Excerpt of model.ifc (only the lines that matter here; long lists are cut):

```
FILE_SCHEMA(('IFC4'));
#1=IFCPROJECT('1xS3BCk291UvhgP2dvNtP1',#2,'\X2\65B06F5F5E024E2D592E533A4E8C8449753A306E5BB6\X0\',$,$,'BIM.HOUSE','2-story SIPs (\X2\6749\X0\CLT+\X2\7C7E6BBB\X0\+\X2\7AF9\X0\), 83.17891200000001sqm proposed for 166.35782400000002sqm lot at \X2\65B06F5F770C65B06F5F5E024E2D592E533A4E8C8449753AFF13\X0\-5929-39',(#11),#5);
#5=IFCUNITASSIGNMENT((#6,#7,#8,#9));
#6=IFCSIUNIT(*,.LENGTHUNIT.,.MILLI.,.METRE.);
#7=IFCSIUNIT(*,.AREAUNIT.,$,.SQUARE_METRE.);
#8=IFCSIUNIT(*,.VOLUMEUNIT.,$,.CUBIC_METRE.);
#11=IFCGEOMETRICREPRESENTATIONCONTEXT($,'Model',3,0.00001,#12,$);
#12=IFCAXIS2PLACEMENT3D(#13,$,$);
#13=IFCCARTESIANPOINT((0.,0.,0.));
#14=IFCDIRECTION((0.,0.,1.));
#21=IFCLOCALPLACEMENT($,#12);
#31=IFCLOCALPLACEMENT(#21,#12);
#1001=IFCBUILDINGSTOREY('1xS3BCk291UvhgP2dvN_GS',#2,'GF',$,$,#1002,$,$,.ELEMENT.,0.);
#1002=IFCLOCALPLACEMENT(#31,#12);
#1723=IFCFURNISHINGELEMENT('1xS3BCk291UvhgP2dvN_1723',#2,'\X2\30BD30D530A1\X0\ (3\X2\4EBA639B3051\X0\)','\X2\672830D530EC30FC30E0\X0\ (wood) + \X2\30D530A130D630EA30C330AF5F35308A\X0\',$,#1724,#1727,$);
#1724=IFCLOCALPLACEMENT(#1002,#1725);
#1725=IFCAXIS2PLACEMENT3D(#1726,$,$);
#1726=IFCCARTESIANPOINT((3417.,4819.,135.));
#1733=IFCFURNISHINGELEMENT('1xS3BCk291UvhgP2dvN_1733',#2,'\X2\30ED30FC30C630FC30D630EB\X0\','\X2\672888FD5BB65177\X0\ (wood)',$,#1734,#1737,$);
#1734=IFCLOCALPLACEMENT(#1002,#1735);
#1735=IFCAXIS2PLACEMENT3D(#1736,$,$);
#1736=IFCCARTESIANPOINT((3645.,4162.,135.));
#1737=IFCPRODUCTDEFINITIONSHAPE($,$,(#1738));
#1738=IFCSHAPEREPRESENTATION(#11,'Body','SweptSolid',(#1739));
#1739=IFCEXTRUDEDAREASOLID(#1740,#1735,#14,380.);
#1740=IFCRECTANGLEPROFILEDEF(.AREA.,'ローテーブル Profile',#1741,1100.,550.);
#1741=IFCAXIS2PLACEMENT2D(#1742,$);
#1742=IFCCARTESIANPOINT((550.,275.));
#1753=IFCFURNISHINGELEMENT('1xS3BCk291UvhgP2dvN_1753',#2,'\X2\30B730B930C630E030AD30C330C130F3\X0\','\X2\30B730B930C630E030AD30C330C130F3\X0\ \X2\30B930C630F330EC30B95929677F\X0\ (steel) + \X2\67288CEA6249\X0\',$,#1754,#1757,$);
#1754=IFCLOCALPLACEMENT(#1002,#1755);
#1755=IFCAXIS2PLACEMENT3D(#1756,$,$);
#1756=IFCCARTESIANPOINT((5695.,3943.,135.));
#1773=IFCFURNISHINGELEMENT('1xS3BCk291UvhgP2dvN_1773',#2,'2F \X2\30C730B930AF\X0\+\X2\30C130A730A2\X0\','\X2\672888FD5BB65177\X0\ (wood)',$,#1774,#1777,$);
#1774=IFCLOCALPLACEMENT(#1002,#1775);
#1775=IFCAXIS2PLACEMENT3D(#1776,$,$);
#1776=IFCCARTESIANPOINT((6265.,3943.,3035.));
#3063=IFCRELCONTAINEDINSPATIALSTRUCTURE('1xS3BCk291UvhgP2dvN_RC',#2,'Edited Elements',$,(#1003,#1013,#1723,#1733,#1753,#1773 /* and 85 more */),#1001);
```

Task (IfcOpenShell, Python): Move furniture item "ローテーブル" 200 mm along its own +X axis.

```python
import ifcopenshell
import ifcopenshell.api.geometry
import ifcopenshell.util.placement

model = ifcopenshell.open("model.ifc")

item = model.by_id(1733)
matrix = ifcopenshell.util.placement.get_local_placement(item.ObjectPlacement)
matrix[:3, 3] += matrix[:3, 0] * 200.0
ifcopenshell.api.geometry.edit_object_placement(model, product=item, matrix=matrix, is_si=False)

print(ifcopenshell.util.placement.get_local_placement(item.ObjectPlacement).round(3) + 0.0)

model.write("model-out.ifc")
```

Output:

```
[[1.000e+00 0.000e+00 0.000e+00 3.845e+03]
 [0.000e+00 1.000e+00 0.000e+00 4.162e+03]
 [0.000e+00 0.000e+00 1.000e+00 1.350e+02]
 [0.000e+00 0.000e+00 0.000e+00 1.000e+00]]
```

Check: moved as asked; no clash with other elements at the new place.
